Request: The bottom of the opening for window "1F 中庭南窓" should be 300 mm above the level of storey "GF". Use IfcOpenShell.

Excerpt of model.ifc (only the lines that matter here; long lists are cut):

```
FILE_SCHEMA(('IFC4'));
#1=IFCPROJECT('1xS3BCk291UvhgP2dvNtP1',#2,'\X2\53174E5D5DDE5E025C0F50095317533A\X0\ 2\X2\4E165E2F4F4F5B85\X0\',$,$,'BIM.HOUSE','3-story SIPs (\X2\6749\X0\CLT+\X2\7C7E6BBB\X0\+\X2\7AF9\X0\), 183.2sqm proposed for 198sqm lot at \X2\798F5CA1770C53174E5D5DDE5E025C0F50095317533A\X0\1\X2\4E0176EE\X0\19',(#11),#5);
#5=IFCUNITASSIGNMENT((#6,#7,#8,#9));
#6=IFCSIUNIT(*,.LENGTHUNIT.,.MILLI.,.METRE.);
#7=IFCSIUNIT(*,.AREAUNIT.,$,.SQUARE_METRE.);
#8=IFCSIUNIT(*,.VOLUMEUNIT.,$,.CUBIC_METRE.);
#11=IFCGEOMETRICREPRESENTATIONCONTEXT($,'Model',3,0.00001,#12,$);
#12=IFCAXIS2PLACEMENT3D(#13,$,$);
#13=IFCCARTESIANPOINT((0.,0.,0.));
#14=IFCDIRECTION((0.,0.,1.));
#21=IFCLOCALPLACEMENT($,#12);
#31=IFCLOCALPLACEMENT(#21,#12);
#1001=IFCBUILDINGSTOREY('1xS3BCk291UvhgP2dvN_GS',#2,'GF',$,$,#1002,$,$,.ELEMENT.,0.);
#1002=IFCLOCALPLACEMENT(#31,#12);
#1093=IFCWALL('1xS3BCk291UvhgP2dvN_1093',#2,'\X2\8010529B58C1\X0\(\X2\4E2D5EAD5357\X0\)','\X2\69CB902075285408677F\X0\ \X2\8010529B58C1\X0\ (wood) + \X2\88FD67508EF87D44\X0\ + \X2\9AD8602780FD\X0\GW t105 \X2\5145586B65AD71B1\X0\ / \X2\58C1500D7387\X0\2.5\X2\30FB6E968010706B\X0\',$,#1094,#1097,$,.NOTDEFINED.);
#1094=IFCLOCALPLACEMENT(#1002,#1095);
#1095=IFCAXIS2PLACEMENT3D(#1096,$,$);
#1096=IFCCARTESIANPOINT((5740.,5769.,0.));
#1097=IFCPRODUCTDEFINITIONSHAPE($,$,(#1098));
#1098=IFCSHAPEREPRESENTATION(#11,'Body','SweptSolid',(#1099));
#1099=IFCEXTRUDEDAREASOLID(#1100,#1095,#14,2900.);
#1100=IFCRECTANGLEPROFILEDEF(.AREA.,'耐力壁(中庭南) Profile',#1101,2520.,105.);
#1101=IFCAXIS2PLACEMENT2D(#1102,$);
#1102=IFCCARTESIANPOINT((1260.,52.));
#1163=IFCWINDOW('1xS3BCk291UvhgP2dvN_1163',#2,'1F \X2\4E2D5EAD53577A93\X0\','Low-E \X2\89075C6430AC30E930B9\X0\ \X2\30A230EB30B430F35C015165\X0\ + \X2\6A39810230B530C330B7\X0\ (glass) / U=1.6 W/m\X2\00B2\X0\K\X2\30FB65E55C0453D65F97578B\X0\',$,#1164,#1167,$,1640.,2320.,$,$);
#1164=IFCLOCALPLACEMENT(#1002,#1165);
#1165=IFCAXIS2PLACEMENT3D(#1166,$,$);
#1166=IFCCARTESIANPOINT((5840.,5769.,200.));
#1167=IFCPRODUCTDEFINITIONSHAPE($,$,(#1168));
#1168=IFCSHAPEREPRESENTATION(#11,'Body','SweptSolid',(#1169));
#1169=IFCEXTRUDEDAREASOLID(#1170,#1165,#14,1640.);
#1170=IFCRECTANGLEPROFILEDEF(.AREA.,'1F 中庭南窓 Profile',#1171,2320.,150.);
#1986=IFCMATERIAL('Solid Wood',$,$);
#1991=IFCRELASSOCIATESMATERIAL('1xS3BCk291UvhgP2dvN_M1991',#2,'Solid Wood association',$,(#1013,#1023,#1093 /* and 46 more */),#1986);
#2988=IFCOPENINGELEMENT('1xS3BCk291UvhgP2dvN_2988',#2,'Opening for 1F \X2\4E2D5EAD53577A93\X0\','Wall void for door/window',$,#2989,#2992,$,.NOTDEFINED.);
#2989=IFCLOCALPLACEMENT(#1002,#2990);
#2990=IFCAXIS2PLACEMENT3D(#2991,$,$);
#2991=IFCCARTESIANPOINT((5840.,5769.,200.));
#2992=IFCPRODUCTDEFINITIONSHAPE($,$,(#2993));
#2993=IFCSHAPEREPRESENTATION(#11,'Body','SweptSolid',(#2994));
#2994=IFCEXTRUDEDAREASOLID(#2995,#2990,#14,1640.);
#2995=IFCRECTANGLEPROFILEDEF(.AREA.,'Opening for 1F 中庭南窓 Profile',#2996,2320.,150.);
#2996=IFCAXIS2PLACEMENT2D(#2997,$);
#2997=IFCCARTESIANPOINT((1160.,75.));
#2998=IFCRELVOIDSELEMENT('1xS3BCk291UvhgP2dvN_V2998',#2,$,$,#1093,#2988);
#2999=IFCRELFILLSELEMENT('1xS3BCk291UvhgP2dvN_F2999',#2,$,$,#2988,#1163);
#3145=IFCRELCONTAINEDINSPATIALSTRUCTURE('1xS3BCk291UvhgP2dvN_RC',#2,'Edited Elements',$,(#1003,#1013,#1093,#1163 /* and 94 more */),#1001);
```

```python
import numpy as np
import ifcopenshell
import ifcopenshell.api.geometry
import ifcopenshell.geom
import ifcopenshell.util.element
import ifcopenshell.util.placement
import ifcopenshell.util.shape
import ifcopenshell.util.unit

model = ifcopenshell.open("model.ifc")
unit_scale = ifcopenshell.util.unit.calculate_unit_scale(model)

window = model.by_guid("1xS3BCk291UvhgP2dvN_1163")
opening = window.FillsVoids[0].RelatingOpeningElement
storey = ifcopenshell.util.element.get_container(window, ifc_class="IfcBuildingStorey")
level = ifcopenshell.util.placement.get_local_placement(storey.ObjectPlacement)[2, 3]

# The opening's origin need not be at the sill, so measure its lowest point.
shape = ifcopenshell.geom.create_shape(ifcopenshell.geom.settings(), opening)
bottom = ifcopenshell.util.shape.get_shape_bottom_elevation(shape, shape.geometry) / unit_scale
dz = level + 0.3 / unit_scale - bottom

shift = np.array([0.0, 0.0, dz])
# The window is not placed relative to its opening, so move both.
for product in (opening, window):
    matrix = ifcopenshell.util.placement.get_local_placement(product.ObjectPlacement)
    matrix[:3, 3] += shift
    ifcopenshell.api.geometry.edit_object_placement(model, product=product, matrix=matrix, is_si=False)

print(f"moved by {dz * unit_scale:+.3f} m")

model.write("model_v2.ifc")
```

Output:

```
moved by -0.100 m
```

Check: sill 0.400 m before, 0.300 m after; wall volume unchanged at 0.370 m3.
